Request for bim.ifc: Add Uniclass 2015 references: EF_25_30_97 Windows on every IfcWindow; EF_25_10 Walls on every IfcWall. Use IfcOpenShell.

First a look at what the model holds.

```python
import ifcopenshell

model = ifcopenshell.open("bim.ifc")
print(model.schema)
print("classifications:", [c.Name for c in model.by_type("IfcClassification")])
for ifc_class in ("IfcDoor", "IfcRoof", "IfcStair", "IfcWall", "IfcWindow"):
    print(ifc_class, len(model.by_type(ifc_class)))
```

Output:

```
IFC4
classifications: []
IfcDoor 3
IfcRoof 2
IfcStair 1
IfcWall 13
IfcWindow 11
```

```python
import ifcopenshell
import ifcopenshell.api.classification

model = ifcopenshell.open("bim.ifc")

system = ifcopenshell.api.classification.add_classification(model, classification="Uniclass 2015")

codes = {
    "IfcWindow": ("EF_25_30_97", "Windows"),
    "IfcWall": ("EF_25_10", "Walls"),
}
for ifc_class, (code, name) in codes.items():
    products = model.by_type(ifc_class)
    ifcopenshell.api.classification.add_reference(
        model, products=products, classification=system, identification=code, name=name
    )
    print(code, len(products))

model.write("bim_v2.ifc")
```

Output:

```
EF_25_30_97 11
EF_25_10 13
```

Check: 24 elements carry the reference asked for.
